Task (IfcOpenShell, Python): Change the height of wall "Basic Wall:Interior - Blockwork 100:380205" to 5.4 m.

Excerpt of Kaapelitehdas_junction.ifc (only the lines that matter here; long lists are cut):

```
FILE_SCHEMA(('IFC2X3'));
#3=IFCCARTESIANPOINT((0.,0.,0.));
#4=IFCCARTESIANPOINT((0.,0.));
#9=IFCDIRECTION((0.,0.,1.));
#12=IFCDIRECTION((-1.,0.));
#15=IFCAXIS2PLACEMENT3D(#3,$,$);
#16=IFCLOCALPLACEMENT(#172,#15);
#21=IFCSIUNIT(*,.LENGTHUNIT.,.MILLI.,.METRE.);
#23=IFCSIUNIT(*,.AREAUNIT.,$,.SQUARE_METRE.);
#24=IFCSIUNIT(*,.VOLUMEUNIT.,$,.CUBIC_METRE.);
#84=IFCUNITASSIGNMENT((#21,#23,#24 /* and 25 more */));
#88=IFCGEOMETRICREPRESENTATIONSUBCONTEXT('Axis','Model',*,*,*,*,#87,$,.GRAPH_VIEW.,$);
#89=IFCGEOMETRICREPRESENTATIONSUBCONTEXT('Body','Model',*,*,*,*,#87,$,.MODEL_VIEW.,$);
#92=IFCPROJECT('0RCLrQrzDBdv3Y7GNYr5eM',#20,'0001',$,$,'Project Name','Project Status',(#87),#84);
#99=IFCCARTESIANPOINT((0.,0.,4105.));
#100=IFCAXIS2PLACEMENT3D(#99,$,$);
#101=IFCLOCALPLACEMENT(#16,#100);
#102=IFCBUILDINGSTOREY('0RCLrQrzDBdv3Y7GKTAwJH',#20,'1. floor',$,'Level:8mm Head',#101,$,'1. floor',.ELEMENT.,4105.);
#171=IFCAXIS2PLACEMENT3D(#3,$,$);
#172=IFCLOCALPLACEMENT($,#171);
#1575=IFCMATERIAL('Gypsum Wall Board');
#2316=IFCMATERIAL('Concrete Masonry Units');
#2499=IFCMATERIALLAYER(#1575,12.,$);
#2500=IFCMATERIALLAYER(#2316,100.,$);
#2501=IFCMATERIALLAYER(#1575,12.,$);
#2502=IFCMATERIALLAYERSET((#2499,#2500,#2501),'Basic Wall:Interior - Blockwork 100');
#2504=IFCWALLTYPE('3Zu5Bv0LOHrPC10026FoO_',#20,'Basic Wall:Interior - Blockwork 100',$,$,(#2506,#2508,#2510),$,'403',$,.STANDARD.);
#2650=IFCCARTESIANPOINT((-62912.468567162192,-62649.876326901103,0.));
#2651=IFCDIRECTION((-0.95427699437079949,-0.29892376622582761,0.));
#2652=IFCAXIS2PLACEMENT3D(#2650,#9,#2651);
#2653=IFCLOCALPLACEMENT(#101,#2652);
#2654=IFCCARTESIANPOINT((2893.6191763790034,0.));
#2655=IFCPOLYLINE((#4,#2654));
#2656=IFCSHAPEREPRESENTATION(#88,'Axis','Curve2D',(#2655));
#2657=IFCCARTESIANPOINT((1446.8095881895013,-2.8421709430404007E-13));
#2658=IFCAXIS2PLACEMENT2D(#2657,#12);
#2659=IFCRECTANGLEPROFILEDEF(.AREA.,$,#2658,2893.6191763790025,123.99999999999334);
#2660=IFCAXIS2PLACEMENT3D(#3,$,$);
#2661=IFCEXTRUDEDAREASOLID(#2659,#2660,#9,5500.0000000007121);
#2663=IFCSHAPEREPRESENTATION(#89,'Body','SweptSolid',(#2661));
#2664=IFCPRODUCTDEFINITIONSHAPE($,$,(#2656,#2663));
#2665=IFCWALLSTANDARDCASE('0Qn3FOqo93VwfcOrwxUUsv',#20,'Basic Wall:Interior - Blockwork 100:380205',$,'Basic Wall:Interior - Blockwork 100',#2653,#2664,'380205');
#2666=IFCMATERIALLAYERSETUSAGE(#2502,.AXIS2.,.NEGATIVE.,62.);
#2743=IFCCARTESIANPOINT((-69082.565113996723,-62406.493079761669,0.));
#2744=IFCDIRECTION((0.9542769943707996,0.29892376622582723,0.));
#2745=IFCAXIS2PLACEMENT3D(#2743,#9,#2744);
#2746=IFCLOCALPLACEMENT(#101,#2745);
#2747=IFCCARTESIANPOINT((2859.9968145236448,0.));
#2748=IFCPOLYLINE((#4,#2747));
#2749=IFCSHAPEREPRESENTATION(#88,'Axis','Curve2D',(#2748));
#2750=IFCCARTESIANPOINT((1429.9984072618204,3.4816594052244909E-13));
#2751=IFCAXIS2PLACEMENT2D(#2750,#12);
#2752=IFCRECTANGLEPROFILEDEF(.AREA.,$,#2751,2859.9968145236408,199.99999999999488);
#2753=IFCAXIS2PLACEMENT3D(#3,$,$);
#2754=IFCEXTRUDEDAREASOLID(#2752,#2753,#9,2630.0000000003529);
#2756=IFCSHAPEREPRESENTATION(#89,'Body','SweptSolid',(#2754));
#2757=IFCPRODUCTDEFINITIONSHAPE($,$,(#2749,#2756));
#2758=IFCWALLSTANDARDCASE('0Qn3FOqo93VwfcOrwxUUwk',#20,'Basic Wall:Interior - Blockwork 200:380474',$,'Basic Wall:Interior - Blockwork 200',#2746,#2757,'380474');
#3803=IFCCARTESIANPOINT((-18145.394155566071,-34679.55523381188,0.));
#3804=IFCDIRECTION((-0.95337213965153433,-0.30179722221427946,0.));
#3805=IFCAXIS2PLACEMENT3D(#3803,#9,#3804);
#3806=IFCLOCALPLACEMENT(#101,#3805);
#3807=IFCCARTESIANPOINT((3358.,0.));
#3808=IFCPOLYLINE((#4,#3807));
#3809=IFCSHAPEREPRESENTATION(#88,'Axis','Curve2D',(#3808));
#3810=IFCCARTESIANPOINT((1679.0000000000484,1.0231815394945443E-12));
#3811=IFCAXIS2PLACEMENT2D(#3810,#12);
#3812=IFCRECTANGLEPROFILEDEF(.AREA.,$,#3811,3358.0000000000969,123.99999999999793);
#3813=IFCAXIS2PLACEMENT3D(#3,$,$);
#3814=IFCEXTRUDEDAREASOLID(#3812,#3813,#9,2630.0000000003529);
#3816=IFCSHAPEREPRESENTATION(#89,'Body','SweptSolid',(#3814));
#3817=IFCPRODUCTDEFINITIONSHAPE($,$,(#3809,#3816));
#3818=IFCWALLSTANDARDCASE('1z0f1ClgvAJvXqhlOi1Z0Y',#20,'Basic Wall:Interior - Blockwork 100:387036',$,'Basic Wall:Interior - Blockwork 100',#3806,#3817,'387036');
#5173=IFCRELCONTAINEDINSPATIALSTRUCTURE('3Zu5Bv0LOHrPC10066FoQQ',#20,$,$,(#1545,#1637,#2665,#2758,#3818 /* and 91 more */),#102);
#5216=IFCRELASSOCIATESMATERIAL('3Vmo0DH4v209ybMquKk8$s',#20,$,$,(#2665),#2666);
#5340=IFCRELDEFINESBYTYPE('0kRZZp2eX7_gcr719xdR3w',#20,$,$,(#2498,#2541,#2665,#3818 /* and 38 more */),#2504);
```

```python
import ifcopenshell
import ifcopenshell.geom
import ifcopenshell.util.representation
import ifcopenshell.util.shape

model = ifcopenshell.open("Kaapelitehdas_junction.ifc")
settings = ifcopenshell.geom.settings()


def volume(element):
    """Net volume in cubic metres, openings subtracted."""
    shape = ifcopenshell.geom.create_shape(settings, element)
    return ifcopenshell.util.shape.get_volume(shape.geometry)


wall = model.by_guid("0Qn3FOqo93VwfcOrwxUUsv")
before = volume(wall)

body = ifcopenshell.util.representation.get_representation(wall, "Model", "Body")
solid = body.Items[0]
old_height = solid.Depth
solid.Depth = 5400.0
after = volume(wall)

print(f"height {old_height:g} -> {solid.Depth:g}, volume {before:.3f} -> {after:.3f} m3")

model.write("Kaapelitehdas_junction_v2.ifc")
```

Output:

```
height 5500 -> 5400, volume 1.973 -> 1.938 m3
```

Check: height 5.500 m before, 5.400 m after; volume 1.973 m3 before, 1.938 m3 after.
